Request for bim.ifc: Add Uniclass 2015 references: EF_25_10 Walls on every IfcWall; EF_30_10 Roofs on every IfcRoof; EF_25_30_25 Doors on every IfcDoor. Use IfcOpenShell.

First a look at what the model holds.

```python
import ifcopenshell

model = ifcopenshell.open("bim.ifc")
print(model.schema)
print("classifications:", [c.Name for c in model.by_type("IfcClassification")])
for ifc_class in ("IfcDoor", "IfcRoof", "IfcStair", "IfcWall", "IfcWindow"):
    print(ifc_class, len(model.by_type(ifc_class)))
```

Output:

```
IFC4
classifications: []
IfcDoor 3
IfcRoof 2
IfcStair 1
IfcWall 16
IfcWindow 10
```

```python
import ifcopenshell
import ifcopenshell.api.classification

model = ifcopenshell.open("bim.ifc")

system = ifcopenshell.api.classification.add_classification(model, classification="Uniclass 2015")

codes = {
    "IfcWall": ("EF_25_10", "Walls"),
    "IfcRoof": ("EF_30_10", "Roofs"),
    "IfcDoor": ("EF_25_30_25", "Doors"),
}
for ifc_class, (code, name) in codes.items():
    products = model.by_type(ifc_class)
    ifcopenshell.api.classification.add_reference(
        model, products=products, classification=system, identification=code, name=name
    )
    print(code, len(products))

model.write("bim-out.ifc")
```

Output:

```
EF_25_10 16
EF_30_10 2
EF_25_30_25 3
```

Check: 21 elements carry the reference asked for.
